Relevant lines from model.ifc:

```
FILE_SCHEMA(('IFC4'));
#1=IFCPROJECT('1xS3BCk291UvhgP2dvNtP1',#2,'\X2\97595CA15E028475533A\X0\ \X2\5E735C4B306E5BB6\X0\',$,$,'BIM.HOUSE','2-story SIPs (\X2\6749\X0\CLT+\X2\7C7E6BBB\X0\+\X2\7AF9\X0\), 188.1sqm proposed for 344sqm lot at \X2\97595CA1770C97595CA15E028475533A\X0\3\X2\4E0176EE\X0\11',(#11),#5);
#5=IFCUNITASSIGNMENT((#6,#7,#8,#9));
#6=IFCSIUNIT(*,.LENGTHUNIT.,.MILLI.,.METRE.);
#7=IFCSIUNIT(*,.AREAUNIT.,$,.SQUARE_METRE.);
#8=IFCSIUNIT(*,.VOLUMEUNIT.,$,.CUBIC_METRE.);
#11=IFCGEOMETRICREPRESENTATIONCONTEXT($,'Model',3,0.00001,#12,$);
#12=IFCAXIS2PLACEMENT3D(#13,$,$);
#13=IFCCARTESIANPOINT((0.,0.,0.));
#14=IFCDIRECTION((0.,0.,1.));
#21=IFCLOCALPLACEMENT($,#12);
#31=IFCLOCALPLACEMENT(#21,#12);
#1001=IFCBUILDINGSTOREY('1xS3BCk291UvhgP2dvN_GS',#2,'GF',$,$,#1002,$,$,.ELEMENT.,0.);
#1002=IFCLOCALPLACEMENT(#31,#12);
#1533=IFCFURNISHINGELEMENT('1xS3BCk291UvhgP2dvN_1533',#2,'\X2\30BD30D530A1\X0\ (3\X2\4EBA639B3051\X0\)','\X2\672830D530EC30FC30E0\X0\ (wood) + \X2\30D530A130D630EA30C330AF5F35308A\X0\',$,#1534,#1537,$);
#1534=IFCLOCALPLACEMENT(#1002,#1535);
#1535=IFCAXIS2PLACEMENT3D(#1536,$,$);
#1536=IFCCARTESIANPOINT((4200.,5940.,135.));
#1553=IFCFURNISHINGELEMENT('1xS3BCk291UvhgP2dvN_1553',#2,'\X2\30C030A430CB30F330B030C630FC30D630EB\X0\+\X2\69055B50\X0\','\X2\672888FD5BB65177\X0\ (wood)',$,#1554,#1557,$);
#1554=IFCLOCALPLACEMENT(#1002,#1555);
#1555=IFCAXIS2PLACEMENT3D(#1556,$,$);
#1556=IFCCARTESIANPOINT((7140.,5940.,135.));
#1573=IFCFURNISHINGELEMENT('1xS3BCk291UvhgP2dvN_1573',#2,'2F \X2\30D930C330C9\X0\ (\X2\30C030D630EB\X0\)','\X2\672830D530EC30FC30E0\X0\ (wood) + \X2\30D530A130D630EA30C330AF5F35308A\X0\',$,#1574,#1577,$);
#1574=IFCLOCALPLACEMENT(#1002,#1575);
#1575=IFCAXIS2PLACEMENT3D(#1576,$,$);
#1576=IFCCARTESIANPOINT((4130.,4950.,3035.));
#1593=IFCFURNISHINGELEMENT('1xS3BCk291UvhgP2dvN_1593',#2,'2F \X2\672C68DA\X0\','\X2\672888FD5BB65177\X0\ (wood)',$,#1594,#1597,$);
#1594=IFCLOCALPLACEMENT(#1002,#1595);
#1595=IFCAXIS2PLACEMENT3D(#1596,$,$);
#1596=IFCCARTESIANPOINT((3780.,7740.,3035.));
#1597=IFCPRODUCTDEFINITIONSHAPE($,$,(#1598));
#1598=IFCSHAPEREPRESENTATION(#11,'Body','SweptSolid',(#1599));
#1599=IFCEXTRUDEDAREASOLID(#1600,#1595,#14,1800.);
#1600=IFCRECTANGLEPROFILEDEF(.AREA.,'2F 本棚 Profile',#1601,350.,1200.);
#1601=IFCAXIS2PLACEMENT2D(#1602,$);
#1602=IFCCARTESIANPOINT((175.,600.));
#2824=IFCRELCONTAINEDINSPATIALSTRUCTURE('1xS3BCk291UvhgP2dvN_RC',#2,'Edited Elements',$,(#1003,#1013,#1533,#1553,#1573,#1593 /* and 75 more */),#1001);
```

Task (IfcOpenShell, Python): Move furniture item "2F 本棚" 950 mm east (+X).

```python
import ifcopenshell
import ifcopenshell.api.geometry
import ifcopenshell.util.placement
import ifcopenshell.util.unit

model = ifcopenshell.open("model.ifc")
unit_scale = ifcopenshell.util.unit.calculate_unit_scale(model)

item = model.by_guid("1xS3BCk291UvhgP2dvN_1593")
matrix = ifcopenshell.util.placement.get_local_placement(item.ObjectPlacement)
matrix[0, 3] += 0.95 / unit_scale
ifcopenshell.api.geometry.edit_object_placement(model, product=item, matrix=matrix, is_si=False)

print(ifcopenshell.util.placement.get_local_placement(item.ObjectPlacement).round(3) + 0.0)

model.write("model_updated.ifc")
```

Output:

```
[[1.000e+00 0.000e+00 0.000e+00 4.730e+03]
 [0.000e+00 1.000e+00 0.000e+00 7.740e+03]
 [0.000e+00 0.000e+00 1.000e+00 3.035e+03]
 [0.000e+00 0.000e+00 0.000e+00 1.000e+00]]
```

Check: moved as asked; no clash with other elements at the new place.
